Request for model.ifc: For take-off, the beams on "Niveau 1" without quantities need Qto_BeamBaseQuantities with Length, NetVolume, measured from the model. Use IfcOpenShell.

First a look at what the model holds.

```python
import ifcopenshell
import ifcopenshell.util.element
import ifcopenshell.util.unit

model = ifcopenshell.open("model.ifc")
print(model.schema)
for unit_type in ("LENGTHUNIT", "AREAUNIT", "VOLUMEUNIT"):
    print(unit_type, ifcopenshell.util.unit.calculate_unit_scale(model, unit_type))
storey = next(s for s in model.by_type("IfcBuildingStorey") if s.Name == "Niveau 1")
beams = [e for e in ifcopenshell.util.element.get_decomposition(storey) if e.is_a("IfcBeam")]
for e in sorted(beams, key=lambda e: e.id()):
    print(e.id(), e.is_a(), e.Name, list(ifcopenshell.util.element.get_psets(e, qtos_only=True)), sep=" | ")
```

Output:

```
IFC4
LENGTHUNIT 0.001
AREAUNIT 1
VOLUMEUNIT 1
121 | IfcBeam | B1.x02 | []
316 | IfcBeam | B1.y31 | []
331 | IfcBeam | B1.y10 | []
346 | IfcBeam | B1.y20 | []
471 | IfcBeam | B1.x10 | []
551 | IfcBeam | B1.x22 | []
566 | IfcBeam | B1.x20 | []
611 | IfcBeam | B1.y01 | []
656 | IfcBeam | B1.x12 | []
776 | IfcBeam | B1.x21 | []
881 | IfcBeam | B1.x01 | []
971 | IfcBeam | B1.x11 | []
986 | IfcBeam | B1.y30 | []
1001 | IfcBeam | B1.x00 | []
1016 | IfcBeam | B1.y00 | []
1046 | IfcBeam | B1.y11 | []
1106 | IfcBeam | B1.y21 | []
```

```python
import ifcopenshell
import ifcopenshell.api.pset
import ifcopenshell.geom
import ifcopenshell.util.element
import ifcopenshell.util.shape
import ifcopenshell.util.unit

model = ifcopenshell.open("model.ifc")
unit_scale = ifcopenshell.util.unit.calculate_unit_scale(model)
volume_scale = ifcopenshell.util.unit.calculate_unit_scale(model, "VOLUMEUNIT")
settings = ifcopenshell.geom.settings()

storey = next(s for s in model.by_type("IfcBuildingStorey") if s.Name == "Niveau 1")
beams = [e for e in ifcopenshell.util.element.get_decomposition(storey) if e.is_a("IfcBeam")]

for e in sorted(beams, key=lambda e: e.id()):
    if ifcopenshell.util.element.get_psets(e, qtos_only=True, should_inherit=False):
        continue
    # Geometry comes back in metres, in the element's own axes.
    shape = ifcopenshell.geom.create_shape(settings, e)
    values = {
        "Length": ifcopenshell.util.shape.get_max_xyz(shape.geometry) / unit_scale,
        "NetVolume": ifcopenshell.util.shape.get_volume(shape.geometry) / volume_scale,
    }
    qto = ifcopenshell.api.pset.add_qto(model, product=e, name="Qto_BeamBaseQuantities")
    ifcopenshell.api.pset.edit_qto(model, qto=qto, properties=values)
    print(e.id(), {k: round(v, 3) for k, v in values.items()})

model.write("model-out.ifc")
```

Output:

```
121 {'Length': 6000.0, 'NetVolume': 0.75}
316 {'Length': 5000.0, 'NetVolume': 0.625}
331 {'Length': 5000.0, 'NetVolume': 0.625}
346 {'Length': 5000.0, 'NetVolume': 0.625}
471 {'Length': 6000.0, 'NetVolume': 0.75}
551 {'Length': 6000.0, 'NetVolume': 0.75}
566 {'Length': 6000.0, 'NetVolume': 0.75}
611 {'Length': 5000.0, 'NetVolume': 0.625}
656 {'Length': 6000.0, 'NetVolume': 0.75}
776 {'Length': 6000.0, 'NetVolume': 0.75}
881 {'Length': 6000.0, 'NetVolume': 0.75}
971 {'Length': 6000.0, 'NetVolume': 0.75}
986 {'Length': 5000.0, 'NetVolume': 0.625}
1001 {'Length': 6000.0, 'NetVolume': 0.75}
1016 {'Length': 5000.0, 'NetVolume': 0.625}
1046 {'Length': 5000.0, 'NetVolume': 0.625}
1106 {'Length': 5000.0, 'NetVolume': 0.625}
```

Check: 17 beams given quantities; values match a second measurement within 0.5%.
